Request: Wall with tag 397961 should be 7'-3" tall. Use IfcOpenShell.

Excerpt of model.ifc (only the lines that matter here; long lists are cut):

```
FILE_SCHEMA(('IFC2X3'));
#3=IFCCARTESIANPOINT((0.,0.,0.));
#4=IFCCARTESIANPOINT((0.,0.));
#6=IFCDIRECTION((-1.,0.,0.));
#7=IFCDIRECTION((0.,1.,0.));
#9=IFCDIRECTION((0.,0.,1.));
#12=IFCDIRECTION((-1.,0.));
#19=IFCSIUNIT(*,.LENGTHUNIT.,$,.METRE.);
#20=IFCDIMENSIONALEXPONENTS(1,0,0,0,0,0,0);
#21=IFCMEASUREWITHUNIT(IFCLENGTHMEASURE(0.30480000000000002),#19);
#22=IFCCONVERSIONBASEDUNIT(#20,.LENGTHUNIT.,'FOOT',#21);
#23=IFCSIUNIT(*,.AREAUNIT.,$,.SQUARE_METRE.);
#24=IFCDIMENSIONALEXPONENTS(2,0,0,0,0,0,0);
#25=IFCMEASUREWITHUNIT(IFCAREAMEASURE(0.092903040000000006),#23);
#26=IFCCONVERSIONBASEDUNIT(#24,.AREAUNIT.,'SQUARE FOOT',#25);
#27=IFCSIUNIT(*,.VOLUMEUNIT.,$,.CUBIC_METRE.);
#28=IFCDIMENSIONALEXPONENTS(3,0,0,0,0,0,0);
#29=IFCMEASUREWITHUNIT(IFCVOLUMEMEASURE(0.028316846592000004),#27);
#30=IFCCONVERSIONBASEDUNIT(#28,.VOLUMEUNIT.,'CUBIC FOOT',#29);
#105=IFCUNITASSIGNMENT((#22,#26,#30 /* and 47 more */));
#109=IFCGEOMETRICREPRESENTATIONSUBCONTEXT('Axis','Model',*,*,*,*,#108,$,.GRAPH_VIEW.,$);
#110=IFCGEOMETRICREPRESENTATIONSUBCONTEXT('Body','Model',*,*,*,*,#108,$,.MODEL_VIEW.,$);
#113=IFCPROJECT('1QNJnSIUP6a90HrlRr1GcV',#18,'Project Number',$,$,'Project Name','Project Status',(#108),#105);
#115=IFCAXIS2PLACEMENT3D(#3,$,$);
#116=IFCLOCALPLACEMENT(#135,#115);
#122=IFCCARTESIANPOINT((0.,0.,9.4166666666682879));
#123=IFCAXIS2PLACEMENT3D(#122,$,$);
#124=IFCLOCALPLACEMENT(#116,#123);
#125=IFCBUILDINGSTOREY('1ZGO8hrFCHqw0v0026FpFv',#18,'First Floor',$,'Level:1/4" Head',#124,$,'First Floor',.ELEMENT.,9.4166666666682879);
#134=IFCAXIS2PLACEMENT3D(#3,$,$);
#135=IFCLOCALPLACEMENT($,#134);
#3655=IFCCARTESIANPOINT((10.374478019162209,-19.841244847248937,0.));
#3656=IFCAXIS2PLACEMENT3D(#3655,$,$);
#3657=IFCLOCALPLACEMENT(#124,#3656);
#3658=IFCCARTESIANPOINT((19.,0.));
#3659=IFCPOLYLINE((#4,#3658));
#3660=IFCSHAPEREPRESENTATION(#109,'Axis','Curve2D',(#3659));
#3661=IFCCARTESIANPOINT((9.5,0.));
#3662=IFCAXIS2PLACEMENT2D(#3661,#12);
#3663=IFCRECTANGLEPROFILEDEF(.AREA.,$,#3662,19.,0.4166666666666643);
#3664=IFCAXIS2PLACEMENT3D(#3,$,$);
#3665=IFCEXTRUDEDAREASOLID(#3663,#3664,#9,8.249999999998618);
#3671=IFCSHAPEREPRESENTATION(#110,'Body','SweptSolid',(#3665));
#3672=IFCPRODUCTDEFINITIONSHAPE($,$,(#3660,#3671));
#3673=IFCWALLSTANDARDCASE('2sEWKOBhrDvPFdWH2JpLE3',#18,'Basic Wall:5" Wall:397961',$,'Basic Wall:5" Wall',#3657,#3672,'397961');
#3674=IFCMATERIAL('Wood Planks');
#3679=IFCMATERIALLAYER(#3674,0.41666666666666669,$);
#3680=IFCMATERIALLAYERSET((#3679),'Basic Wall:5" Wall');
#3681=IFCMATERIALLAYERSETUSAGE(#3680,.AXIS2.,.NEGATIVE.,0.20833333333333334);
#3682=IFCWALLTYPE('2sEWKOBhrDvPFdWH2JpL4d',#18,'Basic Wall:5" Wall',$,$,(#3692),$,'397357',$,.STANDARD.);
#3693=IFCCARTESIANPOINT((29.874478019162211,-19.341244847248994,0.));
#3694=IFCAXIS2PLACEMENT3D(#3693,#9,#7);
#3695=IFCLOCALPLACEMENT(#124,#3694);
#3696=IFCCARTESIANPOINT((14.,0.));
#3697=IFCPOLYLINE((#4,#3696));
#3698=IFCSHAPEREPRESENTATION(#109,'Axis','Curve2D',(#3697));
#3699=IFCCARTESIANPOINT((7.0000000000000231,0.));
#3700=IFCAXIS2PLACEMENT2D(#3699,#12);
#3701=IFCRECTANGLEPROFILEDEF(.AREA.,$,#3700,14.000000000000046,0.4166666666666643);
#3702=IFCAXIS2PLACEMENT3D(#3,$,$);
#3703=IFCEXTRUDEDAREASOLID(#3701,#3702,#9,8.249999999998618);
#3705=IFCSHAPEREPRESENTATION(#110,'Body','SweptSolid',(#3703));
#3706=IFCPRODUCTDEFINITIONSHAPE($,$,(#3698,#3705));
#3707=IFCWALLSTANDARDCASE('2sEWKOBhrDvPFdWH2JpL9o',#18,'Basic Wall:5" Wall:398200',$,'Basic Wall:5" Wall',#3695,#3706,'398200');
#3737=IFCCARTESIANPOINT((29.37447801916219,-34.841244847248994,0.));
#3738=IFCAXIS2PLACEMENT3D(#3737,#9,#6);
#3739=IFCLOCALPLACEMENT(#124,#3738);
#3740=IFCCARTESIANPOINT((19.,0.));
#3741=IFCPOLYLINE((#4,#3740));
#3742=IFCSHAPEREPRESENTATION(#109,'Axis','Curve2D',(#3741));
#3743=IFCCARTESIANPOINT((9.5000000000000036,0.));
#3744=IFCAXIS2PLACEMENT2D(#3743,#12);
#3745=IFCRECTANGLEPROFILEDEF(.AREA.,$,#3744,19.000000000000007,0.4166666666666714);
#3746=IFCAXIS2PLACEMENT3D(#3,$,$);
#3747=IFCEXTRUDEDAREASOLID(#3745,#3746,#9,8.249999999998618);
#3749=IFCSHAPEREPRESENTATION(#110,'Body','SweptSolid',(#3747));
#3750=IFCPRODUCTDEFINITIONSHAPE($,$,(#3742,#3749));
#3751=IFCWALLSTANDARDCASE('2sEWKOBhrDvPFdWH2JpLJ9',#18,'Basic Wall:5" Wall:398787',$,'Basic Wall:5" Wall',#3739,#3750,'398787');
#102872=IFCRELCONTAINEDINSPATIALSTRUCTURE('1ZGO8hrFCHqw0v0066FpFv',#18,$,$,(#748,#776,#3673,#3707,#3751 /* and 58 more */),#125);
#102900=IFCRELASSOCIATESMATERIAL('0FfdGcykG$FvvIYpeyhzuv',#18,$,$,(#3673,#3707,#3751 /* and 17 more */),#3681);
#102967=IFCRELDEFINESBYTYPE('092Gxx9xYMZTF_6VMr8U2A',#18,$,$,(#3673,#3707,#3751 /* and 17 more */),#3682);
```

```python
import ifcopenshell
import ifcopenshell.geom
import ifcopenshell.util.representation
import ifcopenshell.util.shape
import ifcopenshell.util.unit

model = ifcopenshell.open("model.ifc")
unit_scale = ifcopenshell.util.unit.calculate_unit_scale(model)
settings = ifcopenshell.geom.settings()


def volume(element):
    """Net volume in cubic metres, openings subtracted."""
    shape = ifcopenshell.geom.create_shape(settings, element)
    return ifcopenshell.util.shape.get_volume(shape.geometry)


wall = model.by_guid("2sEWKOBhrDvPFdWH2JpLE3")
before = volume(wall)

body = ifcopenshell.util.representation.get_representation(wall, "Model", "Body")
solid = body.Items[0]
old_height = solid.Depth
solid.Depth = 87 * 0.0254 / unit_scale
after = volume(wall)

print(f"height {old_height:g} -> {solid.Depth:g}, volume {before:.3f} -> {after:.3f} m3")

model.write("model_v2.ifc")
```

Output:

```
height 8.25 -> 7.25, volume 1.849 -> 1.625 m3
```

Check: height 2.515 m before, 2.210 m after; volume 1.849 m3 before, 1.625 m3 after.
